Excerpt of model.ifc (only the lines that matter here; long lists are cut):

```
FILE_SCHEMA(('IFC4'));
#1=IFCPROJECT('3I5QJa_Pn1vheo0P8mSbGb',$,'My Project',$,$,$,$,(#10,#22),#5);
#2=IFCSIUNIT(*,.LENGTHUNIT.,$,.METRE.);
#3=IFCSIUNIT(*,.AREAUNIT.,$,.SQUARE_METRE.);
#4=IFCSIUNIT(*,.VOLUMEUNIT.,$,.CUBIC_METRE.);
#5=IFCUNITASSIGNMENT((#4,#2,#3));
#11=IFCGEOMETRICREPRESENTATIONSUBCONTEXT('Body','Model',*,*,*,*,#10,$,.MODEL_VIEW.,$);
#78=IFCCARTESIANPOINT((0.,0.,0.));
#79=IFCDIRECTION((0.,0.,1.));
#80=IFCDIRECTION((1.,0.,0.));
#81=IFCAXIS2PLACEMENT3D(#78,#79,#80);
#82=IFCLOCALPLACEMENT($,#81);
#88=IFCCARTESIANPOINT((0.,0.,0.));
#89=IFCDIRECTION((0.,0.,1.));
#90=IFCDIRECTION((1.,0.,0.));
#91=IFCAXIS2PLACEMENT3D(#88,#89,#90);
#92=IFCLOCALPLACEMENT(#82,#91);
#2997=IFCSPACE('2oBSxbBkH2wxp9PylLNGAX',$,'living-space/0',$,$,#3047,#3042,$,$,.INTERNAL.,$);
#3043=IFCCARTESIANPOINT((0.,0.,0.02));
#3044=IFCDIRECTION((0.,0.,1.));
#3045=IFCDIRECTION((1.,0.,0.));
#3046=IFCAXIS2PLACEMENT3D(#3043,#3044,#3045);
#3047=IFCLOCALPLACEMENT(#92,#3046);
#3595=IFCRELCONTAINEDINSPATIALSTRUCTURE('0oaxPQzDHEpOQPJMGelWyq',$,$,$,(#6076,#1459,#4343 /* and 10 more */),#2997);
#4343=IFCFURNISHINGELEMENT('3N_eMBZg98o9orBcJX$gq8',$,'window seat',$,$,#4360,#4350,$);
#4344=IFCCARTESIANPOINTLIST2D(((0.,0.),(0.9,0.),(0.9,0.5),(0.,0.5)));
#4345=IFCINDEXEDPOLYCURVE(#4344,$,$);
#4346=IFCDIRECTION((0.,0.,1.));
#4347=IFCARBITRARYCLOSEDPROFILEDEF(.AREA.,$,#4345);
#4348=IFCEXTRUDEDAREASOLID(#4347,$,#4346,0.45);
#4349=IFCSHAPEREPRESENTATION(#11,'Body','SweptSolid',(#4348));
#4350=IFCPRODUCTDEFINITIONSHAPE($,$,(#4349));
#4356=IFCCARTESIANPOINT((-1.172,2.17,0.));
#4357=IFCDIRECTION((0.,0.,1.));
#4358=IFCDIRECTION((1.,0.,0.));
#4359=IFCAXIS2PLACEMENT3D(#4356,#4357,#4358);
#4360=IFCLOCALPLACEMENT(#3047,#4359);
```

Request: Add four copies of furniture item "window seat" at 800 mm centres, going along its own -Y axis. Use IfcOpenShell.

```python
import ifcopenshell
import ifcopenshell.api.geometry
import ifcopenshell.api.root
import ifcopenshell.util.element
import ifcopenshell.util.placement
import ifcopenshell.util.unit

model = ifcopenshell.open("model.ifc")
unit_scale = ifcopenshell.util.unit.calculate_unit_scale(model)

source = model.by_guid("3N_eMBZg98o9orBcJX$gq8")
base = ifcopenshell.util.placement.get_local_placement(source.ObjectPlacement)
step = -base[:3, 1] * 0.8 / unit_scale

for i in range(1, 5):
    copy = ifcopenshell.api.root.copy_class(model, product=source)
    copy.Representation = ifcopenshell.util.element.copy_deep(
        model, source.Representation, exclude=["IfcGeometricRepresentationContext", "IfcRepresentationMap"]
    )
    matrix = base.copy()
    matrix[:3, 3] += i * step
    print("added at", matrix[:3, 3].round(3) + 0.0)
    ifcopenshell.api.geometry.edit_object_placement(model, product=copy, matrix=matrix, is_si=False)

model.write("model_edited.ifc")
```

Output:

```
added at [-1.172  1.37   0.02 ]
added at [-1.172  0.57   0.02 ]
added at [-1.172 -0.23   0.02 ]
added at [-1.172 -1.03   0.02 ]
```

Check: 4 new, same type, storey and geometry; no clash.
